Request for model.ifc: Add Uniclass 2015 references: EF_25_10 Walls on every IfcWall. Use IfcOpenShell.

First a look at what the model holds.

```python
import ifcopenshell

model = ifcopenshell.open("model.ifc")
print(model.schema)
print("classifications:", [c.Name for c in model.by_type("IfcClassification")])
for ifc_class in ("IfcDoor", "IfcRoof", "IfcStair", "IfcWall", "IfcWindow"):
    print(ifc_class, len(model.by_type(ifc_class)))
```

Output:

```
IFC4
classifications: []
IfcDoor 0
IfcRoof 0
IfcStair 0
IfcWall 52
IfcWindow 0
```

```python
import ifcopenshell
import ifcopenshell.api.classification

model = ifcopenshell.open("model.ifc")

system = ifcopenshell.api.classification.add_classification(model, classification="Uniclass 2015")

codes = {
    "IfcWall": ("EF_25_10", "Walls"),
}
for ifc_class, (code, name) in codes.items():
    products = model.by_type(ifc_class)
    ifcopenshell.api.classification.add_reference(
        model, products=products, classification=system, identification=code, name=name
    )
    print(code, len(products))

model.write("model_v2.ifc")
```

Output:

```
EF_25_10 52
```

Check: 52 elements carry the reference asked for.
